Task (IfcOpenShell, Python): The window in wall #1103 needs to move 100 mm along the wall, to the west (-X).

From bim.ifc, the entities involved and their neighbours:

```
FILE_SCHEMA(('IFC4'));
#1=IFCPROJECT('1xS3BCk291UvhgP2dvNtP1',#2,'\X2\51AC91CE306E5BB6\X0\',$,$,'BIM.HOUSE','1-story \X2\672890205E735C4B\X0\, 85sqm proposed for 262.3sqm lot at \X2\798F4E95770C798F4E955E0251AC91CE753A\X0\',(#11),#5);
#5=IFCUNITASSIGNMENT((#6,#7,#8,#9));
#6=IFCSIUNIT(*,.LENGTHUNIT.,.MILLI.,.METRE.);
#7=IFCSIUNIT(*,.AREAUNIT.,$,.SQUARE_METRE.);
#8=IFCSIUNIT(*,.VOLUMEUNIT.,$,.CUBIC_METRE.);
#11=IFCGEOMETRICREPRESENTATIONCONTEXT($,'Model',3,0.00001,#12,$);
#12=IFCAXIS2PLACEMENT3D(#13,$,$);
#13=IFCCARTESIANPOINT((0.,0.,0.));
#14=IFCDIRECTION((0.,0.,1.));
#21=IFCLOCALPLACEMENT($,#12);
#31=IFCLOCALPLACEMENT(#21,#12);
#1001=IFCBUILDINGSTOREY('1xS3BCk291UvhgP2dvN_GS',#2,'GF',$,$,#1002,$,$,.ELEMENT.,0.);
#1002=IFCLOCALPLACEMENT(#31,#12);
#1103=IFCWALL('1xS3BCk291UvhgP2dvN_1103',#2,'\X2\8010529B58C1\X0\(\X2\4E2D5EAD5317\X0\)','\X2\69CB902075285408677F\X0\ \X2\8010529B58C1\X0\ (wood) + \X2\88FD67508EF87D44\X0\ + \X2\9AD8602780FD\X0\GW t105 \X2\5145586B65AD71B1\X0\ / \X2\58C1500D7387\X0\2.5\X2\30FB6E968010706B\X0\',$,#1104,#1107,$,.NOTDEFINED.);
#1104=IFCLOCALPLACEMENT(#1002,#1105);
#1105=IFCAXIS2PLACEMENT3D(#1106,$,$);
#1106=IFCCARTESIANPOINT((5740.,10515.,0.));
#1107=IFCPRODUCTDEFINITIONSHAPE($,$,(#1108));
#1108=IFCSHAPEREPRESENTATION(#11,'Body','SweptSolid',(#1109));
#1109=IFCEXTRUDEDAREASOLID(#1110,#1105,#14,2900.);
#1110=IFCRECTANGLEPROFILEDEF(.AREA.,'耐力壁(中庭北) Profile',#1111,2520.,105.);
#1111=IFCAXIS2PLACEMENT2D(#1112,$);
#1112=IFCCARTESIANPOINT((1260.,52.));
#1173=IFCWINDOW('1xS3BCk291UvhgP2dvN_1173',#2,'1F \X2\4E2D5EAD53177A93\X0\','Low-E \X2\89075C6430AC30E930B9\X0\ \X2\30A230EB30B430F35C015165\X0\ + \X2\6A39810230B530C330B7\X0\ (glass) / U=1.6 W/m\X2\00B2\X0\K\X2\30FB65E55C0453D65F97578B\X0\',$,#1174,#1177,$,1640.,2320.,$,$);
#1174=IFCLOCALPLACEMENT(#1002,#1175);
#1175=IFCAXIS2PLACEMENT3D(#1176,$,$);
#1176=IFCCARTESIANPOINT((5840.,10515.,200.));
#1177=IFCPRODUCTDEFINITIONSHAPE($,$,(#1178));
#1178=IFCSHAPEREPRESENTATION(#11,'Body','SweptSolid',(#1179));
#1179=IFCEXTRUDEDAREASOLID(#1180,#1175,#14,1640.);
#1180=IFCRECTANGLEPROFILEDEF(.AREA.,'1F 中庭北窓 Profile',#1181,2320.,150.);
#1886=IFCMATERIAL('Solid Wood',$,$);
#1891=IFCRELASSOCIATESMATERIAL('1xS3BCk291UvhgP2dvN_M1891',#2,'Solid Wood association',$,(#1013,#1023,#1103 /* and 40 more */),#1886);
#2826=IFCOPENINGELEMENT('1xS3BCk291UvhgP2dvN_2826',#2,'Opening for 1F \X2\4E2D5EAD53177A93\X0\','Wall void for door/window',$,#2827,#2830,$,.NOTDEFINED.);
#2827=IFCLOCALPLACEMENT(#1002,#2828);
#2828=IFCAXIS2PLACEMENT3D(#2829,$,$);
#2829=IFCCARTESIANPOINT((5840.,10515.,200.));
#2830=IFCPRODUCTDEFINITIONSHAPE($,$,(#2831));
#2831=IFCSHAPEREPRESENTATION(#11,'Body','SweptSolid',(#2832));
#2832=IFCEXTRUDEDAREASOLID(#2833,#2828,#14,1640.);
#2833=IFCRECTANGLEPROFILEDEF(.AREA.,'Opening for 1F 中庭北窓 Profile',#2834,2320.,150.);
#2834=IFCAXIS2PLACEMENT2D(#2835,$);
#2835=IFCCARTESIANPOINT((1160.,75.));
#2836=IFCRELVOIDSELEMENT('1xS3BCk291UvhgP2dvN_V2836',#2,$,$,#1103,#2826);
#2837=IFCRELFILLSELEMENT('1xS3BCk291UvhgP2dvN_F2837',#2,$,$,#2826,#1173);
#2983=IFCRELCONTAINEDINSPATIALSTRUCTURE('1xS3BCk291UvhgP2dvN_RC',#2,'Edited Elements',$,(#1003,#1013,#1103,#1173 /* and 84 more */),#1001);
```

```python
import ifcopenshell
import ifcopenshell.api.geometry
import ifcopenshell.util.placement

model = ifcopenshell.open("bim.ifc")

window = model.by_guid("1xS3BCk291UvhgP2dvN_1173")
opening = window.FillsVoids[0].RelatingOpeningElement
wall = opening.VoidsElements[0].RelatingBuildingElement

wall_matrix = ifcopenshell.util.placement.get_local_placement(wall.ObjectPlacement)
shift = wall_matrix[:3, 0] * -100.0
before = ifcopenshell.util.placement.get_local_placement(window.ObjectPlacement)[:3, 3].copy()

# The window is not placed relative to its opening, so move both.
for product in (opening, window):
    matrix = ifcopenshell.util.placement.get_local_placement(product.ObjectPlacement)
    matrix[:3, 3] += shift
    ifcopenshell.api.geometry.edit_object_placement(model, product=product, matrix=matrix, is_si=False)

after = ifcopenshell.util.placement.get_local_placement(window.ObjectPlacement)[:3, 3]
print("window moved by", (after - before).round(3) + 0.0)

model.write("bim_rev.ifc")
```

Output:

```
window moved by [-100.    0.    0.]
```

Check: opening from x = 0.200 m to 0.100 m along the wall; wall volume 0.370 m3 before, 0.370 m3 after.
